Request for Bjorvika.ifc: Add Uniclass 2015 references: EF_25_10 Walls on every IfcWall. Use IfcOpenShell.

First a look at what the model holds.

```python
import ifcopenshell

model = ifcopenshell.open("Bjorvika.ifc")
print(model.schema)
print("classifications:", [c.Name for c in model.by_type("IfcClassification")])
for ifc_class in ("IfcDoor", "IfcRoof", "IfcStair", "IfcWall", "IfcWindow"):
    print(ifc_class, len(model.by_type(ifc_class)))
```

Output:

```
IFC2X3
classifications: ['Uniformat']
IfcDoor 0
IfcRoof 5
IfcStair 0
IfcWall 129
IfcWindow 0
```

```python
import ifcopenshell
import ifcopenshell.api.classification

model = ifcopenshell.open("Bjorvika.ifc")

# IFC2X3 requires Source and Edition and has no link from the project to the system.
system = model.create_entity("IfcClassification", Source="NBS", Edition="2015", Name="Uniclass 2015")

codes = {
    "IfcWall": ("EF_25_10", "Walls"),
}
for ifc_class, (code, name) in codes.items():
    products = model.by_type(ifc_class)
    ifcopenshell.api.classification.add_reference(
        model, products=products, classification=system, identification=code, name=name
    )
    print(code, len(products))

model.write("Bjorvika_v2.ifc")
```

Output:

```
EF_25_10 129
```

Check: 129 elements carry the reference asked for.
